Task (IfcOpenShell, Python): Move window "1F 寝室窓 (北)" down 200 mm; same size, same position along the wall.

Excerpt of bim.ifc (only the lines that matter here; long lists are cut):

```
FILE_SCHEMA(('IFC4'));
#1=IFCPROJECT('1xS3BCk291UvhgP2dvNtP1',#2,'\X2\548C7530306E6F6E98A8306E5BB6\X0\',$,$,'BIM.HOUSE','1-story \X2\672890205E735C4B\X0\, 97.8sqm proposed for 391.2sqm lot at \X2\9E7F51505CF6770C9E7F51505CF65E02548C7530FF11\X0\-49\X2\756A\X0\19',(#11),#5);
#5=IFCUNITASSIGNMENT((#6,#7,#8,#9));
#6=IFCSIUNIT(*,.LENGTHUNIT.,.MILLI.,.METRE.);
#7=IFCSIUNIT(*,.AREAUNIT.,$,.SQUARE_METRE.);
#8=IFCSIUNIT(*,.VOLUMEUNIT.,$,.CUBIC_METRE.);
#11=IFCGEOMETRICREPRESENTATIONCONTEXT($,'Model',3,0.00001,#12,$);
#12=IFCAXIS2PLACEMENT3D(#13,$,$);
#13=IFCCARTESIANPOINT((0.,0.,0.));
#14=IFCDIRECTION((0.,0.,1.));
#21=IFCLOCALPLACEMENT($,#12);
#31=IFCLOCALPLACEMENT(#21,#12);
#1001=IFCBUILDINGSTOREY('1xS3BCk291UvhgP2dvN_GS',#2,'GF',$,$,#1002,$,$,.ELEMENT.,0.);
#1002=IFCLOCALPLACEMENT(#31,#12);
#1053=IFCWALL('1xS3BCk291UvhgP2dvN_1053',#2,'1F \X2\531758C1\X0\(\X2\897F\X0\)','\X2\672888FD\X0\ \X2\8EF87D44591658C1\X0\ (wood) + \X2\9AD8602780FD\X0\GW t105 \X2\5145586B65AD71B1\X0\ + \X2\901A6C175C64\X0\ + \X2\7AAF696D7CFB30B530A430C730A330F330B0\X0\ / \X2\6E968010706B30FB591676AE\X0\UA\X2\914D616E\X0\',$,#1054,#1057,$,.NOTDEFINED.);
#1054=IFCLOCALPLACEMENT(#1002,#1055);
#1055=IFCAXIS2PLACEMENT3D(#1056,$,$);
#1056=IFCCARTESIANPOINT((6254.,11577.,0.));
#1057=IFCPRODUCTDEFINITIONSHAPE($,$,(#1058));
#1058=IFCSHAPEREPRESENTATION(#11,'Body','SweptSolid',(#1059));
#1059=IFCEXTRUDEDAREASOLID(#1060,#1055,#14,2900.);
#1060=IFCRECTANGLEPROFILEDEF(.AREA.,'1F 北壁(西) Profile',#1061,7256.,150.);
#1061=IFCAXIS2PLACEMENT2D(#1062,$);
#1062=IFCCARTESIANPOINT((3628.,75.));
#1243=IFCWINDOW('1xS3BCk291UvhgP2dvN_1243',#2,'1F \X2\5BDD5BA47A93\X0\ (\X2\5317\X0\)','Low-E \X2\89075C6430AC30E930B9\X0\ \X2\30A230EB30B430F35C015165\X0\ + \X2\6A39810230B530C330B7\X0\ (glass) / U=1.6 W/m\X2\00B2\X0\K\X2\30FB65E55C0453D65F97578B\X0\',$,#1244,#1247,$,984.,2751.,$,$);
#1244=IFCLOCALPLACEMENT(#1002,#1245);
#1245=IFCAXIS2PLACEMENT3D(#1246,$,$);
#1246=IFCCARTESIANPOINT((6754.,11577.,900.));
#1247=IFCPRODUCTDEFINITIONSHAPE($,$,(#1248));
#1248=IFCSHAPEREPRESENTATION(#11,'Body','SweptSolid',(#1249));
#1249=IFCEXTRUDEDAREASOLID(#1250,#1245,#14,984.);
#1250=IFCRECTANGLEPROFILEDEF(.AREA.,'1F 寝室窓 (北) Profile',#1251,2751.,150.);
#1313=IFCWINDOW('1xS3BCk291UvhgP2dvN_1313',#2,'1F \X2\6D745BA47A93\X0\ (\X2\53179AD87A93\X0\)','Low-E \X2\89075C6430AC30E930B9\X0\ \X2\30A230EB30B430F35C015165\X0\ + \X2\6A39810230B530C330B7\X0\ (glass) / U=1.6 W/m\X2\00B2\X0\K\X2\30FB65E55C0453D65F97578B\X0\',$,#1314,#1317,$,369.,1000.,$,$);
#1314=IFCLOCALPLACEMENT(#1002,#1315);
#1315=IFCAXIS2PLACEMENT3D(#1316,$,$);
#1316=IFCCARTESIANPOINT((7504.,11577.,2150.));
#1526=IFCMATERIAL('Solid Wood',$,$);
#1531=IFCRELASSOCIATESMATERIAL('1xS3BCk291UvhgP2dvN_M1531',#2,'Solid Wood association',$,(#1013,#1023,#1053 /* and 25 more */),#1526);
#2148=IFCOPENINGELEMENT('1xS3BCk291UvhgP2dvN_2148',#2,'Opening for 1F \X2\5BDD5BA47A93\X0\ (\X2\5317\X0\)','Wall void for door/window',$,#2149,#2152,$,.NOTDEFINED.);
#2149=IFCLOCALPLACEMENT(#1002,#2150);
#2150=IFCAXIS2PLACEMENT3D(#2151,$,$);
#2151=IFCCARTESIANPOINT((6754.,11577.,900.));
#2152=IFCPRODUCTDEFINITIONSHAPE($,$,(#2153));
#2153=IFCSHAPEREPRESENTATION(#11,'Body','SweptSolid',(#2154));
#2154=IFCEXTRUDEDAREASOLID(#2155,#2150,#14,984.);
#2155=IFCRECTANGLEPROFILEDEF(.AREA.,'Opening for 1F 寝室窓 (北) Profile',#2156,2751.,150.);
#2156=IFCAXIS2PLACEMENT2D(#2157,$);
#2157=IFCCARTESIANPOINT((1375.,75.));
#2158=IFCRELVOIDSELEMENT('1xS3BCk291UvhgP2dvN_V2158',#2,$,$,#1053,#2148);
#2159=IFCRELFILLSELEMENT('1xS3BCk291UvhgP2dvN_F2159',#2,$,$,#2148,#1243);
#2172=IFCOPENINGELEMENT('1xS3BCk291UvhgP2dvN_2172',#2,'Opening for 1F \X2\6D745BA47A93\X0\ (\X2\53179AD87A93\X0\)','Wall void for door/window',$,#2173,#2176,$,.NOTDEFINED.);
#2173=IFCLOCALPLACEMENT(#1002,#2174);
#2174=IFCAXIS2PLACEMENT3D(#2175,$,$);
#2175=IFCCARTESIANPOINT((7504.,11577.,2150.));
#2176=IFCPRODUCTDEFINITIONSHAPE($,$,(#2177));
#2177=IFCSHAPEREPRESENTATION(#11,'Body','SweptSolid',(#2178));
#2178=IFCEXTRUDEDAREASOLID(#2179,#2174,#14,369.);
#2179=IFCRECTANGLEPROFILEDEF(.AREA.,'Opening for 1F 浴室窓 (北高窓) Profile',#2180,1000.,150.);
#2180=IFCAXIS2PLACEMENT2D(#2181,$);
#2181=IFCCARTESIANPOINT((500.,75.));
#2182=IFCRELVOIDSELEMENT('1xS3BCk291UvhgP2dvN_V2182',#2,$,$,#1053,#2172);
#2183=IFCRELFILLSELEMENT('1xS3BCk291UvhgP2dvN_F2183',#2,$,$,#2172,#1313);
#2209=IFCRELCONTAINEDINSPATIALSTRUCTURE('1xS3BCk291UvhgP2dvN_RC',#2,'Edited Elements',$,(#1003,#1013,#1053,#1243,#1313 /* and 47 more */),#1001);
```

```python
import numpy as np
import ifcopenshell
import ifcopenshell.api.geometry
import ifcopenshell.util.placement
import ifcopenshell.util.unit

model = ifcopenshell.open("bim.ifc")
unit_scale = ifcopenshell.util.unit.calculate_unit_scale(model)

window = model.by_id(1243)
opening = window.FillsVoids[0].RelatingOpeningElement
dz = -0.2 / unit_scale

shift = np.array([0.0, 0.0, dz])
# The window is not placed relative to its opening, so move both.
for product in (opening, window):
    matrix = ifcopenshell.util.placement.get_local_placement(product.ObjectPlacement)
    matrix[:3, 3] += shift
    ifcopenshell.api.geometry.edit_object_placement(model, product=product, matrix=matrix, is_si=False)

print(f"moved by {dz * unit_scale:+.3f} m")

model.write("bim_rev.ifc")
```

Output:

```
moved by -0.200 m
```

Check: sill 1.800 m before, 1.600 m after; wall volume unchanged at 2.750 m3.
